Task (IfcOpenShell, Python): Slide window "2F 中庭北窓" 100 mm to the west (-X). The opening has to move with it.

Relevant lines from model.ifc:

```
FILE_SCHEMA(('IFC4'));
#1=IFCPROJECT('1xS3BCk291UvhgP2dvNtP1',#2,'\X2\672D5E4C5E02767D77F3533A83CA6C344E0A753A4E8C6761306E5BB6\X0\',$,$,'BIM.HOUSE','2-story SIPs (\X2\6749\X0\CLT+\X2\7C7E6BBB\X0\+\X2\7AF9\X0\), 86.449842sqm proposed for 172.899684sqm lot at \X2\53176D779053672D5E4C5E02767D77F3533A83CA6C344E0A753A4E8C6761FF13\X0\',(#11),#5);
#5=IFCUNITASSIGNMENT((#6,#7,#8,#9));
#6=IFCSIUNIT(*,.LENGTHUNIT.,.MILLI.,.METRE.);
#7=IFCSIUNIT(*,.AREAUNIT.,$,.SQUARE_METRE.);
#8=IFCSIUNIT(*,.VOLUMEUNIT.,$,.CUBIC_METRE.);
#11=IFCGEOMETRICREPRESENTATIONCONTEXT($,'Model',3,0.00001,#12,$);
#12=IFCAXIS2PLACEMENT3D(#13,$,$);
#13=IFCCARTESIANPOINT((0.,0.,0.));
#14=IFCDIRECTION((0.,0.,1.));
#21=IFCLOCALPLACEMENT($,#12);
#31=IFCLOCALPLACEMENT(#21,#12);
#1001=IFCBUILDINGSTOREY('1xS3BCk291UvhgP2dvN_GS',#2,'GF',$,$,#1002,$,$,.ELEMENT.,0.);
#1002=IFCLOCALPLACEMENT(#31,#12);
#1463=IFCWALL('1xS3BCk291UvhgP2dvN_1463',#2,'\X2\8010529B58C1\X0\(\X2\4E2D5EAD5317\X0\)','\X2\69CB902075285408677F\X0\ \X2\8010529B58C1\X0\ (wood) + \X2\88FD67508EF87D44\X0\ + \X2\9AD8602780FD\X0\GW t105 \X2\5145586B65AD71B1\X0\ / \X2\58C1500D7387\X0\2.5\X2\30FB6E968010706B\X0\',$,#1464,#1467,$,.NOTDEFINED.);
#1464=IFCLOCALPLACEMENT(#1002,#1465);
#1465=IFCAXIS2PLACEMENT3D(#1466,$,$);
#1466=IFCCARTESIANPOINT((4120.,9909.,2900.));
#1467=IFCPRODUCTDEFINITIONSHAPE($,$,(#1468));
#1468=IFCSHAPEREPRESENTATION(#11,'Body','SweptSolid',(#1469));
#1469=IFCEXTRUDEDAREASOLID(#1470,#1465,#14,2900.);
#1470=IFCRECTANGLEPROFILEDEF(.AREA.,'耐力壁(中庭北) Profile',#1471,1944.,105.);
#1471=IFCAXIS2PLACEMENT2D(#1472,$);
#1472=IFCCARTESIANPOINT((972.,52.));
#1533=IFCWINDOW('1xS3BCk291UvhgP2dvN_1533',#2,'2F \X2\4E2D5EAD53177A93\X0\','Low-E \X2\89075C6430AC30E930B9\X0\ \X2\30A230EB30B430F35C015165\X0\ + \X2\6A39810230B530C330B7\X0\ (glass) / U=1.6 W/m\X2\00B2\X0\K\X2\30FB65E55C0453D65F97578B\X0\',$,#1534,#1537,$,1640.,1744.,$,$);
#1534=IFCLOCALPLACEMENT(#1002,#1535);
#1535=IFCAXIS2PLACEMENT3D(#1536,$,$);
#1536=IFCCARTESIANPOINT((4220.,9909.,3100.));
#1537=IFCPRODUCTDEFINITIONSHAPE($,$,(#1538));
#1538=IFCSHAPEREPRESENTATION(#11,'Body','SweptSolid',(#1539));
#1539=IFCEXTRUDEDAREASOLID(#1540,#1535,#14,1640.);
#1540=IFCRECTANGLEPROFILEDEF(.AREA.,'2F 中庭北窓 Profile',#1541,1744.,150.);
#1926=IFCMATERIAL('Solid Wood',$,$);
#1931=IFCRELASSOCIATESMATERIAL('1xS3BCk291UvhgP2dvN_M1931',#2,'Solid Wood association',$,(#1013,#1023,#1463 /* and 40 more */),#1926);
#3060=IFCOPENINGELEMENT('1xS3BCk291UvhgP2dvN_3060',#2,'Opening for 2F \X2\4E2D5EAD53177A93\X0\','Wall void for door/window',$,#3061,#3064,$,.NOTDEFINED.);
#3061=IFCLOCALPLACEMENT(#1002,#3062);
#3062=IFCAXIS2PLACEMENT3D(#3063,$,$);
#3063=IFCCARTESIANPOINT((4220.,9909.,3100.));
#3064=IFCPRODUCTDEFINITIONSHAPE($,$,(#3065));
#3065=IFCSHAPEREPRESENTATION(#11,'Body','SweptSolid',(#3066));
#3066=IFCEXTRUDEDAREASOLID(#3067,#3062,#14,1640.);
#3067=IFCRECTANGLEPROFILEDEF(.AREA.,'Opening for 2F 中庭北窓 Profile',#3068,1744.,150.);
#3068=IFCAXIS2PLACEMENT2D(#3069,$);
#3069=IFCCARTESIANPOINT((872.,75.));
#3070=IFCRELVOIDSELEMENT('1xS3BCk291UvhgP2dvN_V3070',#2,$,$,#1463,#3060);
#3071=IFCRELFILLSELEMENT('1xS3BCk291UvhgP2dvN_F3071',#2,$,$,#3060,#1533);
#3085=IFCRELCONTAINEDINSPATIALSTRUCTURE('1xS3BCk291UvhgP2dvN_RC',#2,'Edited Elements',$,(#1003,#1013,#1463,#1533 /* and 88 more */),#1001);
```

```python
import ifcopenshell
import ifcopenshell.api.geometry
import ifcopenshell.util.placement

model = ifcopenshell.open("model.ifc")

window = model.by_guid("1xS3BCk291UvhgP2dvN_1533")
opening = window.FillsVoids[0].RelatingOpeningElement
wall = opening.VoidsElements[0].RelatingBuildingElement

wall_matrix = ifcopenshell.util.placement.get_local_placement(wall.ObjectPlacement)
shift = wall_matrix[:3, 0] * -100.0
before = ifcopenshell.util.placement.get_local_placement(window.ObjectPlacement)[:3, 3].copy()

# The window is not placed relative to its opening, so move both.
for product in (opening, window):
    matrix = ifcopenshell.util.placement.get_local_placement(product.ObjectPlacement)
    matrix[:3, 3] += shift
    ifcopenshell.api.geometry.edit_object_placement(model, product=product, matrix=matrix, is_si=False)

after = ifcopenshell.util.placement.get_local_placement(window.ObjectPlacement)[:3, 3]
print("window moved by", (after - before).round(3) + 0.0)

model.write("model-out.ifc")
```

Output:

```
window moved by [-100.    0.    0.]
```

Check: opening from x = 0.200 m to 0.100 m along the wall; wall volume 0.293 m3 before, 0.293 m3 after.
